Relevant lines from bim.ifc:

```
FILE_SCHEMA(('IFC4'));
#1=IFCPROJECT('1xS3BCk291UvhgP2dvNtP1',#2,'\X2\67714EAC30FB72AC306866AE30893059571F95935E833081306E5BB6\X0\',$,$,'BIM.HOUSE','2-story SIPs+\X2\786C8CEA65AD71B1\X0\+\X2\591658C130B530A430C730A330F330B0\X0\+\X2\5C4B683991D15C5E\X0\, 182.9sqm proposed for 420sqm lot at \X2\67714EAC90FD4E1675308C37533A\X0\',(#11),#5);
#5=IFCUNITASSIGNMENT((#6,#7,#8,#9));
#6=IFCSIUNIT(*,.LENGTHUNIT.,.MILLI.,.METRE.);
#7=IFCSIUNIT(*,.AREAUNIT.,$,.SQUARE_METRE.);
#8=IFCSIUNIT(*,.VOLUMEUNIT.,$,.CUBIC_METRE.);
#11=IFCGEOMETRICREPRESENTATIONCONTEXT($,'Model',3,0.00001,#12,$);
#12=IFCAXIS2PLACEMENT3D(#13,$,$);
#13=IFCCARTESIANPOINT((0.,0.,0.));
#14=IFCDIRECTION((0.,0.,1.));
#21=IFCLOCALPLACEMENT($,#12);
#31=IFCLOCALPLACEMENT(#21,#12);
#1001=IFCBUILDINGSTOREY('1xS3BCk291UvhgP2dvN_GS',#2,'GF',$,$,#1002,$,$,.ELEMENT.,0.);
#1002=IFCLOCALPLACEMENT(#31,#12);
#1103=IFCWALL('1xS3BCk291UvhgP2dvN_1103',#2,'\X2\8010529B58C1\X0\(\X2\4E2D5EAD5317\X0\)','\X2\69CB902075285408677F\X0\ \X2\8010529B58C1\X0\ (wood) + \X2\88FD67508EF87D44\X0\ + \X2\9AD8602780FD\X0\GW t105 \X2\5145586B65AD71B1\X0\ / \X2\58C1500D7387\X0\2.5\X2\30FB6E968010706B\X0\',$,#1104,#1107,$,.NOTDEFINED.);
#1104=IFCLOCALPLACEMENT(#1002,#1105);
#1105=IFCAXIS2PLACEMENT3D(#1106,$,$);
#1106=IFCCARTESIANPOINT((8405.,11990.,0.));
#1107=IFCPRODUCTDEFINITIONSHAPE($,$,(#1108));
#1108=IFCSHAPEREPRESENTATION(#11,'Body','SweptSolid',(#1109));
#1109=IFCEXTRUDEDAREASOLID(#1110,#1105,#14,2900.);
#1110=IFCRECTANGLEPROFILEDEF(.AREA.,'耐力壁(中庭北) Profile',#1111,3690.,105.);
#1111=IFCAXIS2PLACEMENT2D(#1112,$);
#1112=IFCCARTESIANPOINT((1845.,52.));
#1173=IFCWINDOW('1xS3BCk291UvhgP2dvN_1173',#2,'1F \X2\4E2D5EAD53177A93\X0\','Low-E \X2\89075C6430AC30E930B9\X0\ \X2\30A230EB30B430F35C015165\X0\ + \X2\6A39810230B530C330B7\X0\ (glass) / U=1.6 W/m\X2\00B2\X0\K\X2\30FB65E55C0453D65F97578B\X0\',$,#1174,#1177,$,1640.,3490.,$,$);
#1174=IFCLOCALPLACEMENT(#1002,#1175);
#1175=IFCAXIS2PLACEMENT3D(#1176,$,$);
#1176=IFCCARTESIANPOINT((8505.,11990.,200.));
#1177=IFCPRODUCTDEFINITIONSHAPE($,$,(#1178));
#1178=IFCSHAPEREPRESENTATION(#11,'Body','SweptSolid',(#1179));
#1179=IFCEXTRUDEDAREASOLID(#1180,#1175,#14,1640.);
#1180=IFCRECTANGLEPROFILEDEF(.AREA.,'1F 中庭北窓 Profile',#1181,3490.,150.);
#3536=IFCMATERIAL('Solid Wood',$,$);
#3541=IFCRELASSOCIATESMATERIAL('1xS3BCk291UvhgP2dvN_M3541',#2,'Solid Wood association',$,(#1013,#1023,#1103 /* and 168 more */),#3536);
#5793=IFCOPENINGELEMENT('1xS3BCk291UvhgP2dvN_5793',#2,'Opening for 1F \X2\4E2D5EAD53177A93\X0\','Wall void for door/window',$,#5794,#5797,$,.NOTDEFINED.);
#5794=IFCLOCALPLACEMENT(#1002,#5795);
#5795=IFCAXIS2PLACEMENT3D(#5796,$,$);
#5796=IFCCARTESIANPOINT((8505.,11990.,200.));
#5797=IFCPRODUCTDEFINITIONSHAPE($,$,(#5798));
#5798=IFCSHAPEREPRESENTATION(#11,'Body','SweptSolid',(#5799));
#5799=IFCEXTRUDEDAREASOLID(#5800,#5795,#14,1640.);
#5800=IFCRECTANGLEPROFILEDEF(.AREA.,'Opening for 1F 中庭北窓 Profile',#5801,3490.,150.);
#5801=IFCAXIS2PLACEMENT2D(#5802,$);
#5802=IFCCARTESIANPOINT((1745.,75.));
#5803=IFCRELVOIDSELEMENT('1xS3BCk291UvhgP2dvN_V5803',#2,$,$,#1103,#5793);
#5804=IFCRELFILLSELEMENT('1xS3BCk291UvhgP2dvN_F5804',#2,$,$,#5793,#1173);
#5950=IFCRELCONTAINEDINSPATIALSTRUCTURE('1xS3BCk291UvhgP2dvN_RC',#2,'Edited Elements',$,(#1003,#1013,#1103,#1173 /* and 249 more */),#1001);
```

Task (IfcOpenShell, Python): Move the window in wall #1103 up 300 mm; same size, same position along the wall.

```python
import numpy as np
import ifcopenshell
import ifcopenshell.api.geometry
import ifcopenshell.util.placement
import ifcopenshell.util.unit

model = ifcopenshell.open("bim.ifc")
unit_scale = ifcopenshell.util.unit.calculate_unit_scale(model)

window = model.by_id(1173)
opening = window.FillsVoids[0].RelatingOpeningElement
dz = 300.0

shift = np.array([0.0, 0.0, dz])
# The window is not placed relative to its opening, so move both.
for product in (opening, window):
    matrix = ifcopenshell.util.placement.get_local_placement(product.ObjectPlacement)
    matrix[:3, 3] += shift
    ifcopenshell.api.geometry.edit_object_placement(model, product=product, matrix=matrix, is_si=False)

print(f"moved by {dz * unit_scale:+.3f} m")

model.write("bim-out.ifc")
```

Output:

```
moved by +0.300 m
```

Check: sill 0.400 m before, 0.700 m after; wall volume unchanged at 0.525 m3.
